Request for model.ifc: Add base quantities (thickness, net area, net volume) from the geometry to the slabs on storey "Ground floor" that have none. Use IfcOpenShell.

First a look at what the model holds.

```python
import ifcopenshell
import ifcopenshell.util.element
import ifcopenshell.util.unit

model = ifcopenshell.open("model.ifc")
print(model.schema)
for unit_type in ("LENGTHUNIT", "AREAUNIT", "VOLUMEUNIT"):
    print(unit_type, ifcopenshell.util.unit.calculate_unit_scale(model, unit_type))
storey = next(s for s in model.by_type("IfcBuildingStorey") if s.Name == "Ground floor")
slabs = [e for e in ifcopenshell.util.element.get_decomposition(storey) if e.is_a("IfcSlab")]
for e in sorted(slabs, key=lambda e: e.id()):
    print(e.id(), e.is_a(), e.Name, list(ifcopenshell.util.element.get_psets(e, qtos_only=True)), sep=" | ")
```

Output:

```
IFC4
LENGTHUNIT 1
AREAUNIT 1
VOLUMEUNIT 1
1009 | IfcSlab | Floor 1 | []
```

```python
import ifcopenshell
import ifcopenshell.api.pset
import ifcopenshell.geom
import ifcopenshell.util.element
import ifcopenshell.util.shape
import ifcopenshell.util.unit

model = ifcopenshell.open("model.ifc")
unit_scale = ifcopenshell.util.unit.calculate_unit_scale(model)
area_scale = ifcopenshell.util.unit.calculate_unit_scale(model, "AREAUNIT")
volume_scale = ifcopenshell.util.unit.calculate_unit_scale(model, "VOLUMEUNIT")
settings = ifcopenshell.geom.settings()

storey = next(s for s in model.by_type("IfcBuildingStorey") if s.Name == "Ground floor")
slabs = [e for e in ifcopenshell.util.element.get_decomposition(storey) if e.is_a("IfcSlab")]

for e in sorted(slabs, key=lambda e: e.id()):
    if ifcopenshell.util.element.get_psets(e, qtos_only=True, should_inherit=False):
        continue
    # Geometry comes back in metres, in the element's own axes.
    shape = ifcopenshell.geom.create_shape(settings, e)
    values = {
        "Width": ifcopenshell.util.shape.get_z(shape.geometry) / unit_scale,
        "NetArea": ifcopenshell.util.shape.get_footprint_area(shape.geometry) / area_scale,
        "NetVolume": ifcopenshell.util.shape.get_volume(shape.geometry) / volume_scale,
    }
    qto = ifcopenshell.api.pset.add_qto(model, product=e, name="Qto_SlabBaseQuantities")
    ifcopenshell.api.pset.edit_qto(model, qto=qto, properties=values)
    print(e.id(), {k: round(v, 3) for k, v in values.items()})

model.write("model_edited.ifc")
```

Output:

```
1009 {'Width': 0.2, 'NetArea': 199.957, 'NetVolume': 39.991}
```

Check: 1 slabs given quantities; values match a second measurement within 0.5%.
